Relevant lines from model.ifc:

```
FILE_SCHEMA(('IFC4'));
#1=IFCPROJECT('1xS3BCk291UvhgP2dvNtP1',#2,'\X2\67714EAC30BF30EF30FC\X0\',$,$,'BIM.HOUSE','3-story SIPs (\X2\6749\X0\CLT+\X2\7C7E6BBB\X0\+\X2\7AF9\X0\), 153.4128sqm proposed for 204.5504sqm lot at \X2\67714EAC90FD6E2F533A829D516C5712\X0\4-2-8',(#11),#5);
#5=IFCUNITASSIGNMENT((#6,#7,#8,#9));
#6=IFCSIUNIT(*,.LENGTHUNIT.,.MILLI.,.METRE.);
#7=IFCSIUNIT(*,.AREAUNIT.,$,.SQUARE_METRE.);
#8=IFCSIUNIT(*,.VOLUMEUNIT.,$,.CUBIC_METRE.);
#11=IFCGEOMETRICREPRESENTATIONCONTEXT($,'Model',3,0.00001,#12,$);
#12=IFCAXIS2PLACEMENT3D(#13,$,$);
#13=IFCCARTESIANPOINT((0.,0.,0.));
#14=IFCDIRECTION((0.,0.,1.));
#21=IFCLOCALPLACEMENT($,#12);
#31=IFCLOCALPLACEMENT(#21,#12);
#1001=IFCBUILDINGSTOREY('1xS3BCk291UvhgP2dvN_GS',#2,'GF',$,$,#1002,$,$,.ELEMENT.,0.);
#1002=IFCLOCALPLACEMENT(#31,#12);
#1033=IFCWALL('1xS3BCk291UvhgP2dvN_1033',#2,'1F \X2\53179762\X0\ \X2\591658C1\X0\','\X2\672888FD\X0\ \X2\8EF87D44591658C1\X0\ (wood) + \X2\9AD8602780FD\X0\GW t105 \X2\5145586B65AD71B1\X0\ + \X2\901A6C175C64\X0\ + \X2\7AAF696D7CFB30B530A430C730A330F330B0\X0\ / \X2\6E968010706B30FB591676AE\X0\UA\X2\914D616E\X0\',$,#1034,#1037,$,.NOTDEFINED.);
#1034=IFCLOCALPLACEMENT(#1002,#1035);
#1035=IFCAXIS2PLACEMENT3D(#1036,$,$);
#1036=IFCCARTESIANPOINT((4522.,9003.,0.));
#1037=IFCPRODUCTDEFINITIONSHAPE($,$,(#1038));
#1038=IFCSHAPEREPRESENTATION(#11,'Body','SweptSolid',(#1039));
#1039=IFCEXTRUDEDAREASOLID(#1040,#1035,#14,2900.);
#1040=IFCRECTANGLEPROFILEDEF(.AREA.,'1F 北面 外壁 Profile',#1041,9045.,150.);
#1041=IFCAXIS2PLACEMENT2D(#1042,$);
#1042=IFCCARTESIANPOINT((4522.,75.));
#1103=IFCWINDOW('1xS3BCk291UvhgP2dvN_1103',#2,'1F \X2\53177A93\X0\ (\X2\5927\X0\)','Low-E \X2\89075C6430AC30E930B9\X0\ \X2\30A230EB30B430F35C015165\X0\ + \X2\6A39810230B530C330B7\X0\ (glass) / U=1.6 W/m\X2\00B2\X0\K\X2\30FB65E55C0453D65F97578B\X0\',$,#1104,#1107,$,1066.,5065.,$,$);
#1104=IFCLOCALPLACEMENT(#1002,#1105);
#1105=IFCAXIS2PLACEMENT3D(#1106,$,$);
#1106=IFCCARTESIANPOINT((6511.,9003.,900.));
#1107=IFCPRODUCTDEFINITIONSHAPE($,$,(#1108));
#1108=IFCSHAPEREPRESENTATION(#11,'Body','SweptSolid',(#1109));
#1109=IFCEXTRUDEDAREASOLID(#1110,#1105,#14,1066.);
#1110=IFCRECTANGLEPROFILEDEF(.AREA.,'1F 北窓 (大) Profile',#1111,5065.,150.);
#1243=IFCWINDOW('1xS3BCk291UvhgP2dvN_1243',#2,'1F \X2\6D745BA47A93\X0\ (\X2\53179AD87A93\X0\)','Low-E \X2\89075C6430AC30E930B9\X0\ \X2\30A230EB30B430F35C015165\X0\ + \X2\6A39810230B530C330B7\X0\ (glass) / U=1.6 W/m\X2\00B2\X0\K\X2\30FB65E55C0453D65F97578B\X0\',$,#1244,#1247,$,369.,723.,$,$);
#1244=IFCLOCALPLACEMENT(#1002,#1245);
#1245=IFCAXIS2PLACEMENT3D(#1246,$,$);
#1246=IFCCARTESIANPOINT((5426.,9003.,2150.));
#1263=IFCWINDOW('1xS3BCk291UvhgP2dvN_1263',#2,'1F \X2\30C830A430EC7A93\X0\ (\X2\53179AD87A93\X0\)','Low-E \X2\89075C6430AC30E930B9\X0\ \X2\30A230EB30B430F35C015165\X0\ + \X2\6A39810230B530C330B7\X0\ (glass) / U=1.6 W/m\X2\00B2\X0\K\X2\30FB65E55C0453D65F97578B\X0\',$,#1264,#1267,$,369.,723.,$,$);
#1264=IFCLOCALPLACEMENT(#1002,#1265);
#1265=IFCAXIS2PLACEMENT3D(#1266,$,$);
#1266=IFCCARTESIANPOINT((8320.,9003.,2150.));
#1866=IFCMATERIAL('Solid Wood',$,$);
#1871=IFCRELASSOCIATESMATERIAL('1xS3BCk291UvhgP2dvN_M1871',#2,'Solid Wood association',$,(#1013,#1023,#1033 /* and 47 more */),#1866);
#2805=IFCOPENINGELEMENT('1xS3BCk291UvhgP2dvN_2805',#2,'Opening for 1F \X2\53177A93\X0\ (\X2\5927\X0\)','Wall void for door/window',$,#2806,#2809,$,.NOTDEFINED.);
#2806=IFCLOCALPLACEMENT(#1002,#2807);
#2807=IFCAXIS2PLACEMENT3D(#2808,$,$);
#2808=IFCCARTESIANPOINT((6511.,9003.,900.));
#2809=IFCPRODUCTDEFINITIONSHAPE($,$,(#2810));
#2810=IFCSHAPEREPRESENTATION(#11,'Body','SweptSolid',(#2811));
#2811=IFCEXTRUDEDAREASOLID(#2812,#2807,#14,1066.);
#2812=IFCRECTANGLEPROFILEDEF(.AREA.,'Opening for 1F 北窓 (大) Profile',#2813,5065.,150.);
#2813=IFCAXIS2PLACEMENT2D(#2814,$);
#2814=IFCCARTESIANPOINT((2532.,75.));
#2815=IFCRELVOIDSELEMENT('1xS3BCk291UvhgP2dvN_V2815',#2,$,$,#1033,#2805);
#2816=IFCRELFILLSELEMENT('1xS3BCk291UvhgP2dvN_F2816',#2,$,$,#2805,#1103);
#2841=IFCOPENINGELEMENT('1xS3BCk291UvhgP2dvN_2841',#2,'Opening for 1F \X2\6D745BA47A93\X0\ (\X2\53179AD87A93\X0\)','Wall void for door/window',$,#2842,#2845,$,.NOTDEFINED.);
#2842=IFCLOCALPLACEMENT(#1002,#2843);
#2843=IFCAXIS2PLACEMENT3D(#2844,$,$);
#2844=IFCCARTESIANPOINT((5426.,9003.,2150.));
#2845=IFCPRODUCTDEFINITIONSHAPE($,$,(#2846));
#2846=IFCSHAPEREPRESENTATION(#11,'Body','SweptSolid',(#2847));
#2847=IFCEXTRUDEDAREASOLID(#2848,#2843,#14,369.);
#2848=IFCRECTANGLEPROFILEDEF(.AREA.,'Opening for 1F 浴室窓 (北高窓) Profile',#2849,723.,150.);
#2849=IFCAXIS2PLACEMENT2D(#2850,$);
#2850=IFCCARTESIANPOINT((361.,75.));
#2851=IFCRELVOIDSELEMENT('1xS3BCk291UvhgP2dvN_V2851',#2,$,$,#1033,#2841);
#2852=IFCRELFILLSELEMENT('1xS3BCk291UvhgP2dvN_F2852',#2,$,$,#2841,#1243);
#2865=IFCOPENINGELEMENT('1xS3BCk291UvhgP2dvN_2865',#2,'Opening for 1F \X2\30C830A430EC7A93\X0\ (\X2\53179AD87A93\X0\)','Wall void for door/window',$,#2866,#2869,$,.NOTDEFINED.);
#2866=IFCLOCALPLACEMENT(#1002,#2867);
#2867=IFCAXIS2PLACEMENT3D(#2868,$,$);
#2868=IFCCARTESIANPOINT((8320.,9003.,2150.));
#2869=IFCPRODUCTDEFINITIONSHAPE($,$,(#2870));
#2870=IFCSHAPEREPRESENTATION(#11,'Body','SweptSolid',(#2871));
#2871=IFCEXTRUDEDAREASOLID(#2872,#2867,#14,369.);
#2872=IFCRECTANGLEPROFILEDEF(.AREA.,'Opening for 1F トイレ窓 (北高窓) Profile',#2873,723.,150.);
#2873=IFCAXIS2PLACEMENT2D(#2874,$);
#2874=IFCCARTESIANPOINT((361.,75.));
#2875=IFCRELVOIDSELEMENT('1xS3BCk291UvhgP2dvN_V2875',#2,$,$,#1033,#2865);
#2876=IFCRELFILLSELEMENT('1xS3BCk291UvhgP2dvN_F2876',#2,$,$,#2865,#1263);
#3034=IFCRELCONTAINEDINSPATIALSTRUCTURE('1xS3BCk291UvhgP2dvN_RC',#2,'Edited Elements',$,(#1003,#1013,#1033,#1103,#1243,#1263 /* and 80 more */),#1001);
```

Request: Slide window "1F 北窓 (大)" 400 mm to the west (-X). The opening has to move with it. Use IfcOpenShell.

```python
import ifcopenshell
import ifcopenshell.api.geometry
import ifcopenshell.util.placement
import ifcopenshell.util.unit

model = ifcopenshell.open("model.ifc")
unit_scale = ifcopenshell.util.unit.calculate_unit_scale(model)

window = model.by_id(1103)
opening = window.FillsVoids[0].RelatingOpeningElement
wall = opening.VoidsElements[0].RelatingBuildingElement

wall_matrix = ifcopenshell.util.placement.get_local_placement(wall.ObjectPlacement)
shift = wall_matrix[:3, 0] * -0.4 / unit_scale
before = ifcopenshell.util.placement.get_local_placement(window.ObjectPlacement)[:3, 3].copy()

# The window is not placed relative to its opening, so move both.
for product in (opening, window):
    matrix = ifcopenshell.util.placement.get_local_placement(product.ObjectPlacement)
    matrix[:3, 3] += shift
    ifcopenshell.api.geometry.edit_object_placement(model, product=product, matrix=matrix, is_si=False)

after = ifcopenshell.util.placement.get_local_placement(window.ObjectPlacement)[:3, 3]
print("window moved by", (after - before).round(3) + 0.0)

model.write("model-out.ifc")
```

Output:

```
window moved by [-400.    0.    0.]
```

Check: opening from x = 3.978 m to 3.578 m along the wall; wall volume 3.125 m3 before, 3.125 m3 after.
